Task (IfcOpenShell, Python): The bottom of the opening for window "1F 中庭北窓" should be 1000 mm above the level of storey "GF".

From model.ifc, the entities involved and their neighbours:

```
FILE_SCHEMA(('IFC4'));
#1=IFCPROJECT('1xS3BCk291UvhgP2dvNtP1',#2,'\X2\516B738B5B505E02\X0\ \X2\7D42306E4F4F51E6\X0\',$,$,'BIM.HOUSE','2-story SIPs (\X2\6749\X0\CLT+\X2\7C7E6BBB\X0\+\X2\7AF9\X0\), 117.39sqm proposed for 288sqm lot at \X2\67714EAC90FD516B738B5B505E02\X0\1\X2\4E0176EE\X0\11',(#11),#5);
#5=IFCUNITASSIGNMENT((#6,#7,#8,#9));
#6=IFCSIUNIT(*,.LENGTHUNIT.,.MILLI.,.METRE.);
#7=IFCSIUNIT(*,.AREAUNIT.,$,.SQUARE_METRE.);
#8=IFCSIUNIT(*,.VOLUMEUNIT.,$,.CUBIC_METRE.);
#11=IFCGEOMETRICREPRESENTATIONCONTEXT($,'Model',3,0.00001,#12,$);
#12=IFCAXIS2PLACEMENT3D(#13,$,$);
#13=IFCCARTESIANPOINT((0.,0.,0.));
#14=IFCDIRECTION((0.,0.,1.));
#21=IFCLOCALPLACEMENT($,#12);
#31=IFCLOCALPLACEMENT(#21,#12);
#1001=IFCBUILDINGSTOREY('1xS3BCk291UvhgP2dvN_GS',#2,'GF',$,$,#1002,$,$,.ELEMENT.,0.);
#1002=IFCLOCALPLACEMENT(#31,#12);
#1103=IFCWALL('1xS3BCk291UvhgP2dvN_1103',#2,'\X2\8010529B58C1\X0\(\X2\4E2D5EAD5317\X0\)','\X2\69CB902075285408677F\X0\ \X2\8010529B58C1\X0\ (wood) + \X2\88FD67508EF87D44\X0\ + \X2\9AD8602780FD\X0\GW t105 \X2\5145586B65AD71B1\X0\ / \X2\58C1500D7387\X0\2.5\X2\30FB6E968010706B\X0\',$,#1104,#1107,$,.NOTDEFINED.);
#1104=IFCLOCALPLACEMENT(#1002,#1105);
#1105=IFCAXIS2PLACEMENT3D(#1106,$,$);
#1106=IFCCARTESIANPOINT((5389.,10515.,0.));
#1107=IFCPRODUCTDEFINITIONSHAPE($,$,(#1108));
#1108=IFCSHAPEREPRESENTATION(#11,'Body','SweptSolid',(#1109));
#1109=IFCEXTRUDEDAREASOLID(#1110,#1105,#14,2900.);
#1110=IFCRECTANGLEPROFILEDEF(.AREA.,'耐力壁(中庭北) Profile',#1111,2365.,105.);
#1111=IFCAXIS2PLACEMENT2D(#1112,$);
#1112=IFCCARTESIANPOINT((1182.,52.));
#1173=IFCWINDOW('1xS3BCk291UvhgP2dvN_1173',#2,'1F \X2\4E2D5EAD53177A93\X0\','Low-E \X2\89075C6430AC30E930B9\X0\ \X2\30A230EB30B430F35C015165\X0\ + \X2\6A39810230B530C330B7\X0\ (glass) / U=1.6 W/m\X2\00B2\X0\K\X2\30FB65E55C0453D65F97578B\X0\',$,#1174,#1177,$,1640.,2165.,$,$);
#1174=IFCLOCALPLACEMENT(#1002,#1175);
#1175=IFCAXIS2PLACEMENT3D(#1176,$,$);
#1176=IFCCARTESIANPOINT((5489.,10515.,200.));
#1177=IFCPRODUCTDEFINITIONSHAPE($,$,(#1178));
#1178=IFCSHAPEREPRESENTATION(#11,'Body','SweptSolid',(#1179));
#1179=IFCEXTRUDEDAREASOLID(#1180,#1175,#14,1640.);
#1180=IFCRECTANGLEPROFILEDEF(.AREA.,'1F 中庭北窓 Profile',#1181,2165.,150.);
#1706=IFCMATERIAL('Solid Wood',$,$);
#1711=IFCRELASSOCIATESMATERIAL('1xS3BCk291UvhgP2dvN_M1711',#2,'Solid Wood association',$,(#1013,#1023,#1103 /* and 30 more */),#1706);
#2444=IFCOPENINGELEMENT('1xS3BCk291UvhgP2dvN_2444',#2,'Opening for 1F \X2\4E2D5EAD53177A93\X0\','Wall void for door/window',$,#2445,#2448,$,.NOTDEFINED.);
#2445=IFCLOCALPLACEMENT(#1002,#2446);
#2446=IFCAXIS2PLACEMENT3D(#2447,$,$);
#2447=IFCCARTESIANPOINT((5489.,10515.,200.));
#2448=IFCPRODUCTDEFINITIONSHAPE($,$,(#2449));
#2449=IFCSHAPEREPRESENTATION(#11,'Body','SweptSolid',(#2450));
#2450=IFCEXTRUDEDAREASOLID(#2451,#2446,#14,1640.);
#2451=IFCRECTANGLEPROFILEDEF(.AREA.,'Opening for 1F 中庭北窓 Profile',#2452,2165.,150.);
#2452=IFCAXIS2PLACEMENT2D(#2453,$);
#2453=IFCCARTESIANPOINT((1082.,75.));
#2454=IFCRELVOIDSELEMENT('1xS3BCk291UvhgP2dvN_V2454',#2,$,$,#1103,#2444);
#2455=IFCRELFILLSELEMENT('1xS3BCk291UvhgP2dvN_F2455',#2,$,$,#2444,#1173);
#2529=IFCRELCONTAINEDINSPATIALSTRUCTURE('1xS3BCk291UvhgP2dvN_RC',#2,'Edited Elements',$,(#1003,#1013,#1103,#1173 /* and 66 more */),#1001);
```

```python
import numpy as np
import ifcopenshell
import ifcopenshell.api.geometry
import ifcopenshell.geom
import ifcopenshell.util.element
import ifcopenshell.util.placement
import ifcopenshell.util.shape
import ifcopenshell.util.unit

model = ifcopenshell.open("model.ifc")
unit_scale = ifcopenshell.util.unit.calculate_unit_scale(model)

window = model.by_guid("1xS3BCk291UvhgP2dvN_1173")
opening = window.FillsVoids[0].RelatingOpeningElement
storey = ifcopenshell.util.element.get_container(window, ifc_class="IfcBuildingStorey")
level = ifcopenshell.util.placement.get_local_placement(storey.ObjectPlacement)[2, 3]

# The opening's origin need not be at the sill, so measure its lowest point.
shape = ifcopenshell.geom.create_shape(ifcopenshell.geom.settings(), opening)
bottom = ifcopenshell.util.shape.get_shape_bottom_elevation(shape, shape.geometry) / unit_scale
dz = level + 1000.0 - bottom

shift = np.array([0.0, 0.0, dz])
# The window is not placed relative to its opening, so move both.
for product in (opening, window):
    matrix = ifcopenshell.util.placement.get_local_placement(product.ObjectPlacement)
    matrix[:3, 3] += shift
    ifcopenshell.api.geometry.edit_object_placement(model, product=product, matrix=matrix, is_si=False)

print(f"moved by {dz * unit_scale:+.3f} m")

model.write("model_edited.ifc")
```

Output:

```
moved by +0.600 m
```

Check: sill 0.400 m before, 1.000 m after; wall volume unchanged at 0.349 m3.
